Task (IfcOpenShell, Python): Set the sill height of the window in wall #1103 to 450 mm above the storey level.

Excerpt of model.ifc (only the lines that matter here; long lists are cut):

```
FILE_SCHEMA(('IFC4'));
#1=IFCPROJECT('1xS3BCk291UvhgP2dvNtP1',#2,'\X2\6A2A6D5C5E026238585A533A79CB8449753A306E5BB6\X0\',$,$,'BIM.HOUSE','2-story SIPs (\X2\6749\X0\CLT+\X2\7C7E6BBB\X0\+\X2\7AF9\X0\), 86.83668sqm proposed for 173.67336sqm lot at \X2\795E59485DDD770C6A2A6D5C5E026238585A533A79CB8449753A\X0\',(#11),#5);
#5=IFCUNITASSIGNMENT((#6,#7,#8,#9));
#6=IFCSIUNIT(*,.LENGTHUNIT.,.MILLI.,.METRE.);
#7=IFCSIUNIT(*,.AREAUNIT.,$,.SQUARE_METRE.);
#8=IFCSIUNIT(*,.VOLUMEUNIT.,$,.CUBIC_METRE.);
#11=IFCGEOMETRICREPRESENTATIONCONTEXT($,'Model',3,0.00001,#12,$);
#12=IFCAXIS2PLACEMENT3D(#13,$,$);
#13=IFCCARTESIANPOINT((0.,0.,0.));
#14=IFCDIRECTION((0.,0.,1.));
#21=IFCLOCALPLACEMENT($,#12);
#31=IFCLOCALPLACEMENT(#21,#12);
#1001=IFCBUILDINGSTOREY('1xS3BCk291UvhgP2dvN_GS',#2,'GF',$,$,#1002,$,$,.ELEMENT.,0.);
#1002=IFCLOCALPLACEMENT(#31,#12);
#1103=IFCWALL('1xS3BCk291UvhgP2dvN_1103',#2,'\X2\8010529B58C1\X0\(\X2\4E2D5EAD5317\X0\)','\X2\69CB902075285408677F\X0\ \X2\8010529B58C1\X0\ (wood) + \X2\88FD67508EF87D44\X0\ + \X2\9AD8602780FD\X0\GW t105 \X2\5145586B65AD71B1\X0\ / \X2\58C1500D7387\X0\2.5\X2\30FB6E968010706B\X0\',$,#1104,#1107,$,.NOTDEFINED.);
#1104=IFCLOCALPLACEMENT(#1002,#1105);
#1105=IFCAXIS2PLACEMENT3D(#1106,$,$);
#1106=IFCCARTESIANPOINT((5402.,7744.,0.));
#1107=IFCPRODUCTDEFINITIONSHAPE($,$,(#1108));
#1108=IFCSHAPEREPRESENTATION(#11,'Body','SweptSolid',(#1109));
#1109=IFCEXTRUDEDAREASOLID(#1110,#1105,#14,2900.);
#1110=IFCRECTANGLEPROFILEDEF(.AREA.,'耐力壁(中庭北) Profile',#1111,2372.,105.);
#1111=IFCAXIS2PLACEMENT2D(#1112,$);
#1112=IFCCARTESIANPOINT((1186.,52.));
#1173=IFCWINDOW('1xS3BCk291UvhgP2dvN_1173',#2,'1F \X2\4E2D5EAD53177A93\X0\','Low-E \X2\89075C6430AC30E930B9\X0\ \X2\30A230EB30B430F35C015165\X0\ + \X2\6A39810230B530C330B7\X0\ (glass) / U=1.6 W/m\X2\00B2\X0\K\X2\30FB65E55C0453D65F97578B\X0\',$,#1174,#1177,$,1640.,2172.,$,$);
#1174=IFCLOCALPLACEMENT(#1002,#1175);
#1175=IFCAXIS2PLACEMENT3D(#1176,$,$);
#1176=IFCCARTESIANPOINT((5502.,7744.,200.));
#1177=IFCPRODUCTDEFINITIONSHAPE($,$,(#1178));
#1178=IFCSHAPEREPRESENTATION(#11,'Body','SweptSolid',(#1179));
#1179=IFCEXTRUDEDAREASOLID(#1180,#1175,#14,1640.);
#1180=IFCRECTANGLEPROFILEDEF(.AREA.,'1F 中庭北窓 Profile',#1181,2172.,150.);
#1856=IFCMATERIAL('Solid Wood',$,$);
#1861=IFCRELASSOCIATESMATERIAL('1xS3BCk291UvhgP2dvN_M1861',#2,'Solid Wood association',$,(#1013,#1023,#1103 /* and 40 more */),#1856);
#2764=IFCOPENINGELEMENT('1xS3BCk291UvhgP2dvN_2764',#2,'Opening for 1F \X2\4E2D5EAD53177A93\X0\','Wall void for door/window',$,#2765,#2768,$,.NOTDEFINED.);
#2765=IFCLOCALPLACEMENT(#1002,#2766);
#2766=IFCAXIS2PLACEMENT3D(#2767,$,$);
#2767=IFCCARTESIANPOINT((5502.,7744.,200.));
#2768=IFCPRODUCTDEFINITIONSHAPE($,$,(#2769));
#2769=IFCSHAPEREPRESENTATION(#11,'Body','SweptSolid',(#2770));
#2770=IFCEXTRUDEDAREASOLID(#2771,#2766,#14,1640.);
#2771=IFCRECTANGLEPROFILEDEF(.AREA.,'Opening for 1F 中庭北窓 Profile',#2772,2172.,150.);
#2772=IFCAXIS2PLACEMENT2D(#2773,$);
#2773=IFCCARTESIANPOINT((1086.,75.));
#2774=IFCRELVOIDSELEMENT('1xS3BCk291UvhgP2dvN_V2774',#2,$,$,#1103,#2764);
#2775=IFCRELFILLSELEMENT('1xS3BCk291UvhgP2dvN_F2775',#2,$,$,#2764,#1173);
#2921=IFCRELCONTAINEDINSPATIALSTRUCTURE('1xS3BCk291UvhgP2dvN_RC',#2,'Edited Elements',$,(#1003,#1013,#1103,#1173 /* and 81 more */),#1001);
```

```python
import numpy as np
import ifcopenshell
import ifcopenshell.api.geometry
import ifcopenshell.geom
import ifcopenshell.util.element
import ifcopenshell.util.placement
import ifcopenshell.util.shape
import ifcopenshell.util.unit

model = ifcopenshell.open("model.ifc")
unit_scale = ifcopenshell.util.unit.calculate_unit_scale(model)

window = model.by_id(1173)
opening = window.FillsVoids[0].RelatingOpeningElement
storey = ifcopenshell.util.element.get_container(window, ifc_class="IfcBuildingStorey")
level = ifcopenshell.util.placement.get_local_placement(storey.ObjectPlacement)[2, 3]

# The opening's origin need not be at the sill, so measure its lowest point.
shape = ifcopenshell.geom.create_shape(ifcopenshell.geom.settings(), opening)
bottom = ifcopenshell.util.shape.get_shape_bottom_elevation(shape, shape.geometry) / unit_scale
dz = level + 0.45 / unit_scale - bottom

shift = np.array([0.0, 0.0, dz])
# The window is not placed relative to its opening, so move both.
for product in (opening, window):
    matrix = ifcopenshell.util.placement.get_local_placement(product.ObjectPlacement)
    matrix[:3, 3] += shift
    ifcopenshell.api.geometry.edit_object_placement(model, product=product, matrix=matrix, is_si=False)

print(f"moved by {dz * unit_scale:+.3f} m")

model.write("model_v2.ifc")
```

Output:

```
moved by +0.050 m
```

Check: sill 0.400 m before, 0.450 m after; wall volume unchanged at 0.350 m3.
